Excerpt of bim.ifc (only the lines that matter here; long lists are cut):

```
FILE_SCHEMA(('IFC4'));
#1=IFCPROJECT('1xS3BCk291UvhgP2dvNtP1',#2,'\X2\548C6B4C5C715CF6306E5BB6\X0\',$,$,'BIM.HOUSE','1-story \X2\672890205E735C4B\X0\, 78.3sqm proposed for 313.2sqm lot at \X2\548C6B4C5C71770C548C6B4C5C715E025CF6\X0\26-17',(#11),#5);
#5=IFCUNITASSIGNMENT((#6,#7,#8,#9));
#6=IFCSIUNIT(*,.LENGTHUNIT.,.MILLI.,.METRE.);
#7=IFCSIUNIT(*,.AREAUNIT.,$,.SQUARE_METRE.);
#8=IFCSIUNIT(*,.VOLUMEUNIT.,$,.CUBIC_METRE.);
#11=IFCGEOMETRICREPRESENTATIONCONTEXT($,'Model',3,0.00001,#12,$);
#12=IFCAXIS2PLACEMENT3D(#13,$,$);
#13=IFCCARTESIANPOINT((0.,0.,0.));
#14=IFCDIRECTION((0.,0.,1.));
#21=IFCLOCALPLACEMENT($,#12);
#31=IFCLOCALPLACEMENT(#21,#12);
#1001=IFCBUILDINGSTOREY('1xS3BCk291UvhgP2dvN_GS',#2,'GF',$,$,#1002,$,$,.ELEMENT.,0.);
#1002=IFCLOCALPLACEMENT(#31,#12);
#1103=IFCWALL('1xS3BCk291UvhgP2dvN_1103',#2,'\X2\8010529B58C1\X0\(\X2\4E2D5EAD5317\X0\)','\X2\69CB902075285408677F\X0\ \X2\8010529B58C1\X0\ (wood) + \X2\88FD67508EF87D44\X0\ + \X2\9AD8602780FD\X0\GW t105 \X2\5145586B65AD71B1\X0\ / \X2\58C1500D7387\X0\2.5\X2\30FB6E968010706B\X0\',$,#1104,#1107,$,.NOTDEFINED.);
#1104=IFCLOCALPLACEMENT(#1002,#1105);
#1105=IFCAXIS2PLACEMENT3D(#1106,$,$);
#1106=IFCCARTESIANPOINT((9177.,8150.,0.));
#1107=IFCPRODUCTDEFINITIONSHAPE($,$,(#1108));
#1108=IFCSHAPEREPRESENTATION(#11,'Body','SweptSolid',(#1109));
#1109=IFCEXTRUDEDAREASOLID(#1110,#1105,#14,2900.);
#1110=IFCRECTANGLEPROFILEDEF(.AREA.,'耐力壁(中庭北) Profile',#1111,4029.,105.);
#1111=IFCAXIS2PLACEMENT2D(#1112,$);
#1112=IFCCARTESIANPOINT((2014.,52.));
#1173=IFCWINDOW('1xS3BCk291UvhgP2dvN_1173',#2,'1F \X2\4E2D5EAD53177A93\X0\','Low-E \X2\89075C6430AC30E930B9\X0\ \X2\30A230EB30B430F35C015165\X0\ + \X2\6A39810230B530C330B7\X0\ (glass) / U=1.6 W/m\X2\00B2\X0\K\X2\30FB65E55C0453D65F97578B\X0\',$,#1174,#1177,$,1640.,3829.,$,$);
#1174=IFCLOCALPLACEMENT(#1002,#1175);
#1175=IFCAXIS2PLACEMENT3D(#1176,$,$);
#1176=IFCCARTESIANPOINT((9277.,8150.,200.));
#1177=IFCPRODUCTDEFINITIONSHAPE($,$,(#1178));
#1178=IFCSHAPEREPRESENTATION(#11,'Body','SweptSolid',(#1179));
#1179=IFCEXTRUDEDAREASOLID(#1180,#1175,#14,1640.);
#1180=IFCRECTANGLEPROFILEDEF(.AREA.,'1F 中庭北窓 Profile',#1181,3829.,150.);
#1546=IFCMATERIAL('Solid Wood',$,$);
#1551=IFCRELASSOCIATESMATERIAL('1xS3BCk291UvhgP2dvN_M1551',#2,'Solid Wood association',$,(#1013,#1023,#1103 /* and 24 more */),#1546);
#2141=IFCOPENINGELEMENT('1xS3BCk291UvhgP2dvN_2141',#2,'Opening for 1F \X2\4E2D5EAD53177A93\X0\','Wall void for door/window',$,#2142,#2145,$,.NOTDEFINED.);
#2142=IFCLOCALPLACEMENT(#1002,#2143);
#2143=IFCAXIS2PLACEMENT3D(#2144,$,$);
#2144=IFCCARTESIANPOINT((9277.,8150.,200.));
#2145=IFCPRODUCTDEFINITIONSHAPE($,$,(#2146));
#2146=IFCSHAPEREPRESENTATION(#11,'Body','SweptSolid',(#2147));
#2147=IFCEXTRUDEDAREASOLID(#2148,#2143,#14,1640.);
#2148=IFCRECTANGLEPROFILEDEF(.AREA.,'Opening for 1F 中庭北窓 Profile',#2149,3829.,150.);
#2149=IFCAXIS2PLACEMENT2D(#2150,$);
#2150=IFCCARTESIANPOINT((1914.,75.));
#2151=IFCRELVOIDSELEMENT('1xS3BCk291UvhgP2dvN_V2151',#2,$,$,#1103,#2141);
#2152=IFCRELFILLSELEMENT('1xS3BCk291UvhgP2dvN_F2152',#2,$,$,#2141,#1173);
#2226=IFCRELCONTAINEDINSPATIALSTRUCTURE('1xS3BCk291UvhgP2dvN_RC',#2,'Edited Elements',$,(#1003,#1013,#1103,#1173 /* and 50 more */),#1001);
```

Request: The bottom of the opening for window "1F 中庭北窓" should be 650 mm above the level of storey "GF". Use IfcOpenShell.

```python
import numpy as np
import ifcopenshell
import ifcopenshell.api.geometry
import ifcopenshell.geom
import ifcopenshell.util.element
import ifcopenshell.util.placement
import ifcopenshell.util.shape
import ifcopenshell.util.unit

model = ifcopenshell.open("bim.ifc")
unit_scale = ifcopenshell.util.unit.calculate_unit_scale(model)

window = model.by_id(1173)
opening = window.FillsVoids[0].RelatingOpeningElement
storey = ifcopenshell.util.element.get_container(window, ifc_class="IfcBuildingStorey")
level = ifcopenshell.util.placement.get_local_placement(storey.ObjectPlacement)[2, 3]

# The opening's origin need not be at the sill, so measure its lowest point.
shape = ifcopenshell.geom.create_shape(ifcopenshell.geom.settings(), opening)
bottom = ifcopenshell.util.shape.get_shape_bottom_elevation(shape, shape.geometry) / unit_scale
dz = level + 0.65 / unit_scale - bottom

shift = np.array([0.0, 0.0, dz])
# The window is not placed relative to its opening, so move both.
for product in (opening, window):
    matrix = ifcopenshell.util.placement.get_local_placement(product.ObjectPlacement)
    matrix[:3, 3] += shift
    ifcopenshell.api.geometry.edit_object_placement(model, product=product, matrix=matrix, is_si=False)

print(f"moved by {dz * unit_scale:+.3f} m")

model.write("bim_updated.ifc")
```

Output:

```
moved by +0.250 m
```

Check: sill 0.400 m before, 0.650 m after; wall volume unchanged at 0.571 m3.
